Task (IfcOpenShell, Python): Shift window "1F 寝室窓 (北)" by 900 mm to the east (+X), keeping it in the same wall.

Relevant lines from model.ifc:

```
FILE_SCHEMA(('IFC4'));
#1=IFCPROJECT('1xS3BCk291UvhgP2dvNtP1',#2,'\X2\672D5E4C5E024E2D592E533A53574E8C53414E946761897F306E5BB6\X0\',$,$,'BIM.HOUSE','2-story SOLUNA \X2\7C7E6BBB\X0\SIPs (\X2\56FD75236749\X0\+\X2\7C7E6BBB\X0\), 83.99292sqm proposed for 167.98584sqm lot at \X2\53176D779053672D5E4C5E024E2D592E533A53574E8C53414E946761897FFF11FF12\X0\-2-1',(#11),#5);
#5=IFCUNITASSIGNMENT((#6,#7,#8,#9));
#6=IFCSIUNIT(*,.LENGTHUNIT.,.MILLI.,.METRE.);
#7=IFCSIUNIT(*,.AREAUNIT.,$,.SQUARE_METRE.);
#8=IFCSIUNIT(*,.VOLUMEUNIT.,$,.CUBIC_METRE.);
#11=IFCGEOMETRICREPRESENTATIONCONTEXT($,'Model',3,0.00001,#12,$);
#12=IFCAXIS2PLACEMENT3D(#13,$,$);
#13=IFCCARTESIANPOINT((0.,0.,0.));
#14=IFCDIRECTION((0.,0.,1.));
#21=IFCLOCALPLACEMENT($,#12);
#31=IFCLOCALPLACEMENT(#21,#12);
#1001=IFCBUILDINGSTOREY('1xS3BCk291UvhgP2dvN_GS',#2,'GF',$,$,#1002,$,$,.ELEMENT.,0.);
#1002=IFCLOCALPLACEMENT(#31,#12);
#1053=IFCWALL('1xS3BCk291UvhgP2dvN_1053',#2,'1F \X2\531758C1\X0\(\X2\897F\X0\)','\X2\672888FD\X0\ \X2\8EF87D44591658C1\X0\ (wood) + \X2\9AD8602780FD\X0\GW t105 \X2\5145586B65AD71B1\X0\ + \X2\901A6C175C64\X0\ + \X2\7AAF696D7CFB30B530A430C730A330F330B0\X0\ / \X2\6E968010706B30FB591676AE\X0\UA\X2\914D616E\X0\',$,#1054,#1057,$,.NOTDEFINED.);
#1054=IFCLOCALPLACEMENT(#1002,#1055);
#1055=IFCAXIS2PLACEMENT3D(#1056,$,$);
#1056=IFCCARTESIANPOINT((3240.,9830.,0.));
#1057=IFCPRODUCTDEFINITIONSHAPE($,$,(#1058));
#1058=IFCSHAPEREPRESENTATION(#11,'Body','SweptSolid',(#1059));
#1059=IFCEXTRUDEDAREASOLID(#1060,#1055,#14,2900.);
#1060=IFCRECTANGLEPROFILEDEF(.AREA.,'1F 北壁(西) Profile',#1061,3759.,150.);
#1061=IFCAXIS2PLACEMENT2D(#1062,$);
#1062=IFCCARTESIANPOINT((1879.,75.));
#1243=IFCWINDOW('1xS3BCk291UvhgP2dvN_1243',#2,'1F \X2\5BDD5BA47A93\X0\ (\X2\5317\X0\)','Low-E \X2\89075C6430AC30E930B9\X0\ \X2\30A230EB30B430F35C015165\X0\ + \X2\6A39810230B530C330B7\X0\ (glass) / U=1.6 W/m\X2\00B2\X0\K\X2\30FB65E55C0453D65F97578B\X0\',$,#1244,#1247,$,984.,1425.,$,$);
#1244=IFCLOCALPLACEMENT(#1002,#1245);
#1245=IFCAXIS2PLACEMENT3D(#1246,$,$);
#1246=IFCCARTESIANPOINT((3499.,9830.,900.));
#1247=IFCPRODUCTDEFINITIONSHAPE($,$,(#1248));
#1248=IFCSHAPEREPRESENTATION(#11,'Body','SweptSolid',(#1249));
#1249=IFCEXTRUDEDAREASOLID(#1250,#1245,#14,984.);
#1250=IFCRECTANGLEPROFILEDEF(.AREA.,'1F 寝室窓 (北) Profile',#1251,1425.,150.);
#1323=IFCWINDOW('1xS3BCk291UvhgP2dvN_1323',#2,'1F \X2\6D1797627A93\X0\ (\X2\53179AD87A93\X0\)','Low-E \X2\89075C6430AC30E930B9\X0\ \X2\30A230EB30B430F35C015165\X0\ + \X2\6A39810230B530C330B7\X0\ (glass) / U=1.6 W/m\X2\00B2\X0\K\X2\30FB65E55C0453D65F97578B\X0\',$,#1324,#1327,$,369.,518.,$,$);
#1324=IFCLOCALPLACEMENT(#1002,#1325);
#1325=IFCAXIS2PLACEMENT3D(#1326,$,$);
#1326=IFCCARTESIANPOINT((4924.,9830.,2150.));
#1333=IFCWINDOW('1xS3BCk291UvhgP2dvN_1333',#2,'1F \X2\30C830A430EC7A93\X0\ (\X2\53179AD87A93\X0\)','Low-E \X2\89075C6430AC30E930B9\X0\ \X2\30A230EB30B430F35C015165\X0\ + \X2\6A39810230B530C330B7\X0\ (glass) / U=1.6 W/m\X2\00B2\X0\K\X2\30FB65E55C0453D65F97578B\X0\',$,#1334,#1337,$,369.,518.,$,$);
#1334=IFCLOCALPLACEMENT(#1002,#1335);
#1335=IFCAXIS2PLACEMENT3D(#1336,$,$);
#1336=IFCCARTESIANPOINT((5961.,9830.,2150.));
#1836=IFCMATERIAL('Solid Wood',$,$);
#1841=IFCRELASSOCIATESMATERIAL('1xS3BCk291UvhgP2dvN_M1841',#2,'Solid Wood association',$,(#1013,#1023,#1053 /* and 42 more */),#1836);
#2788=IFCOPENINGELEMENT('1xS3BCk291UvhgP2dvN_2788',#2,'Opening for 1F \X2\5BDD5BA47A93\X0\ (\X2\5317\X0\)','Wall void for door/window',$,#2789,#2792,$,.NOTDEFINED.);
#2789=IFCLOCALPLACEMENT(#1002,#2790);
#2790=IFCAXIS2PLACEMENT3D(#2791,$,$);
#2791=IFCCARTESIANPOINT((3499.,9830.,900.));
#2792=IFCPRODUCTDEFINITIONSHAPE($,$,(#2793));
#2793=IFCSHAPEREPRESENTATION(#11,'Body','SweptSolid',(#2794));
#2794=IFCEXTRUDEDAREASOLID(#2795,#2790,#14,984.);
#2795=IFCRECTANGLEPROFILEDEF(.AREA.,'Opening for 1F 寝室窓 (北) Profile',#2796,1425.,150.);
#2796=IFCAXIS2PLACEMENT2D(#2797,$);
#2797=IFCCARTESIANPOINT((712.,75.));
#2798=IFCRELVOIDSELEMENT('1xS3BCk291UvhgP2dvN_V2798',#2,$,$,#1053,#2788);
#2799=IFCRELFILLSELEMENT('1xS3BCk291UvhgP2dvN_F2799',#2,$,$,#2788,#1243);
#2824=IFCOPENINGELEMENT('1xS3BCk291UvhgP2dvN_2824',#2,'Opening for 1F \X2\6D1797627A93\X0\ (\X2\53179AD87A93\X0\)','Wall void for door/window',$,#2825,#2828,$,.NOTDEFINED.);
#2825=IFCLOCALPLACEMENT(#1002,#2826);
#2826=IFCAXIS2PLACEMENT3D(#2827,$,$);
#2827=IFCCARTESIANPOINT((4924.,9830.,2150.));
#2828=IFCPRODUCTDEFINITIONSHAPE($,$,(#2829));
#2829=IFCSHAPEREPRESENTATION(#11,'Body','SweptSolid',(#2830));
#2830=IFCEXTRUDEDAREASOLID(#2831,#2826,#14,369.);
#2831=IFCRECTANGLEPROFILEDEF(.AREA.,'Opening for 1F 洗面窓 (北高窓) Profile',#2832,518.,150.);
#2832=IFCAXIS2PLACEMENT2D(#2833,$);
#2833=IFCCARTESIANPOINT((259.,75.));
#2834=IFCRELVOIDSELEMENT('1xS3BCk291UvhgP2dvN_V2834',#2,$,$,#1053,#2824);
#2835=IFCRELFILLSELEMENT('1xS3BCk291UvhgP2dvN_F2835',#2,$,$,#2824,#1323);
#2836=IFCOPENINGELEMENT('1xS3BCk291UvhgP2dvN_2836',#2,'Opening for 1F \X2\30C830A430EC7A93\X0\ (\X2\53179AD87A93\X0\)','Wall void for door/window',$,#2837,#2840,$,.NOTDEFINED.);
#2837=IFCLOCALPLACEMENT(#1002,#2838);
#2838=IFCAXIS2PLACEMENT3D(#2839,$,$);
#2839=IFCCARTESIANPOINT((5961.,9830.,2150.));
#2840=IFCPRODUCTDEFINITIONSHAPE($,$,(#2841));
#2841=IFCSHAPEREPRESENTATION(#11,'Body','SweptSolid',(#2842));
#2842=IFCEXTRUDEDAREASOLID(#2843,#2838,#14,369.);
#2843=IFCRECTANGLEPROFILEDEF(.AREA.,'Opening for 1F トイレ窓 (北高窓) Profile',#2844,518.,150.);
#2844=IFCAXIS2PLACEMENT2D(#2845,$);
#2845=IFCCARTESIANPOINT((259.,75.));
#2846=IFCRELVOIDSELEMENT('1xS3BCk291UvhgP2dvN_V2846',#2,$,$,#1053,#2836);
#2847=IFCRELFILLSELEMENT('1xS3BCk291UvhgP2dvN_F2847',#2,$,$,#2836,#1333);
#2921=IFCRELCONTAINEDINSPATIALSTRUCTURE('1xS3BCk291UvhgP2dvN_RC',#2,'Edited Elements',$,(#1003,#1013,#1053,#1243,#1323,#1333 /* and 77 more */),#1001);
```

```python
import ifcopenshell
import ifcopenshell.api.geometry
import ifcopenshell.util.placement
import ifcopenshell.util.unit

model = ifcopenshell.open("model.ifc")
unit_scale = ifcopenshell.util.unit.calculate_unit_scale(model)

window = model.by_guid("1xS3BCk291UvhgP2dvN_1243")
opening = window.FillsVoids[0].RelatingOpeningElement
wall = opening.VoidsElements[0].RelatingBuildingElement

wall_matrix = ifcopenshell.util.placement.get_local_placement(wall.ObjectPlacement)
shift = wall_matrix[:3, 0] * 0.9 / unit_scale
before = ifcopenshell.util.placement.get_local_placement(window.ObjectPlacement)[:3, 3].copy()

# The window is not placed relative to its opening, so move both.
for product in (opening, window):
    matrix = ifcopenshell.util.placement.get_local_placement(product.ObjectPlacement)
    matrix[:3, 3] += shift
    ifcopenshell.api.geometry.edit_object_placement(model, product=product, matrix=matrix, is_si=False)

after = ifcopenshell.util.placement.get_local_placement(window.ObjectPlacement)[:3, 3]
print("window moved by", (after - before).round(3) + 0.0)

model.write("model_rev.ifc")
```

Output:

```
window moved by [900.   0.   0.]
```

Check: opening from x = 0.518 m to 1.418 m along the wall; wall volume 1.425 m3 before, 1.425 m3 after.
